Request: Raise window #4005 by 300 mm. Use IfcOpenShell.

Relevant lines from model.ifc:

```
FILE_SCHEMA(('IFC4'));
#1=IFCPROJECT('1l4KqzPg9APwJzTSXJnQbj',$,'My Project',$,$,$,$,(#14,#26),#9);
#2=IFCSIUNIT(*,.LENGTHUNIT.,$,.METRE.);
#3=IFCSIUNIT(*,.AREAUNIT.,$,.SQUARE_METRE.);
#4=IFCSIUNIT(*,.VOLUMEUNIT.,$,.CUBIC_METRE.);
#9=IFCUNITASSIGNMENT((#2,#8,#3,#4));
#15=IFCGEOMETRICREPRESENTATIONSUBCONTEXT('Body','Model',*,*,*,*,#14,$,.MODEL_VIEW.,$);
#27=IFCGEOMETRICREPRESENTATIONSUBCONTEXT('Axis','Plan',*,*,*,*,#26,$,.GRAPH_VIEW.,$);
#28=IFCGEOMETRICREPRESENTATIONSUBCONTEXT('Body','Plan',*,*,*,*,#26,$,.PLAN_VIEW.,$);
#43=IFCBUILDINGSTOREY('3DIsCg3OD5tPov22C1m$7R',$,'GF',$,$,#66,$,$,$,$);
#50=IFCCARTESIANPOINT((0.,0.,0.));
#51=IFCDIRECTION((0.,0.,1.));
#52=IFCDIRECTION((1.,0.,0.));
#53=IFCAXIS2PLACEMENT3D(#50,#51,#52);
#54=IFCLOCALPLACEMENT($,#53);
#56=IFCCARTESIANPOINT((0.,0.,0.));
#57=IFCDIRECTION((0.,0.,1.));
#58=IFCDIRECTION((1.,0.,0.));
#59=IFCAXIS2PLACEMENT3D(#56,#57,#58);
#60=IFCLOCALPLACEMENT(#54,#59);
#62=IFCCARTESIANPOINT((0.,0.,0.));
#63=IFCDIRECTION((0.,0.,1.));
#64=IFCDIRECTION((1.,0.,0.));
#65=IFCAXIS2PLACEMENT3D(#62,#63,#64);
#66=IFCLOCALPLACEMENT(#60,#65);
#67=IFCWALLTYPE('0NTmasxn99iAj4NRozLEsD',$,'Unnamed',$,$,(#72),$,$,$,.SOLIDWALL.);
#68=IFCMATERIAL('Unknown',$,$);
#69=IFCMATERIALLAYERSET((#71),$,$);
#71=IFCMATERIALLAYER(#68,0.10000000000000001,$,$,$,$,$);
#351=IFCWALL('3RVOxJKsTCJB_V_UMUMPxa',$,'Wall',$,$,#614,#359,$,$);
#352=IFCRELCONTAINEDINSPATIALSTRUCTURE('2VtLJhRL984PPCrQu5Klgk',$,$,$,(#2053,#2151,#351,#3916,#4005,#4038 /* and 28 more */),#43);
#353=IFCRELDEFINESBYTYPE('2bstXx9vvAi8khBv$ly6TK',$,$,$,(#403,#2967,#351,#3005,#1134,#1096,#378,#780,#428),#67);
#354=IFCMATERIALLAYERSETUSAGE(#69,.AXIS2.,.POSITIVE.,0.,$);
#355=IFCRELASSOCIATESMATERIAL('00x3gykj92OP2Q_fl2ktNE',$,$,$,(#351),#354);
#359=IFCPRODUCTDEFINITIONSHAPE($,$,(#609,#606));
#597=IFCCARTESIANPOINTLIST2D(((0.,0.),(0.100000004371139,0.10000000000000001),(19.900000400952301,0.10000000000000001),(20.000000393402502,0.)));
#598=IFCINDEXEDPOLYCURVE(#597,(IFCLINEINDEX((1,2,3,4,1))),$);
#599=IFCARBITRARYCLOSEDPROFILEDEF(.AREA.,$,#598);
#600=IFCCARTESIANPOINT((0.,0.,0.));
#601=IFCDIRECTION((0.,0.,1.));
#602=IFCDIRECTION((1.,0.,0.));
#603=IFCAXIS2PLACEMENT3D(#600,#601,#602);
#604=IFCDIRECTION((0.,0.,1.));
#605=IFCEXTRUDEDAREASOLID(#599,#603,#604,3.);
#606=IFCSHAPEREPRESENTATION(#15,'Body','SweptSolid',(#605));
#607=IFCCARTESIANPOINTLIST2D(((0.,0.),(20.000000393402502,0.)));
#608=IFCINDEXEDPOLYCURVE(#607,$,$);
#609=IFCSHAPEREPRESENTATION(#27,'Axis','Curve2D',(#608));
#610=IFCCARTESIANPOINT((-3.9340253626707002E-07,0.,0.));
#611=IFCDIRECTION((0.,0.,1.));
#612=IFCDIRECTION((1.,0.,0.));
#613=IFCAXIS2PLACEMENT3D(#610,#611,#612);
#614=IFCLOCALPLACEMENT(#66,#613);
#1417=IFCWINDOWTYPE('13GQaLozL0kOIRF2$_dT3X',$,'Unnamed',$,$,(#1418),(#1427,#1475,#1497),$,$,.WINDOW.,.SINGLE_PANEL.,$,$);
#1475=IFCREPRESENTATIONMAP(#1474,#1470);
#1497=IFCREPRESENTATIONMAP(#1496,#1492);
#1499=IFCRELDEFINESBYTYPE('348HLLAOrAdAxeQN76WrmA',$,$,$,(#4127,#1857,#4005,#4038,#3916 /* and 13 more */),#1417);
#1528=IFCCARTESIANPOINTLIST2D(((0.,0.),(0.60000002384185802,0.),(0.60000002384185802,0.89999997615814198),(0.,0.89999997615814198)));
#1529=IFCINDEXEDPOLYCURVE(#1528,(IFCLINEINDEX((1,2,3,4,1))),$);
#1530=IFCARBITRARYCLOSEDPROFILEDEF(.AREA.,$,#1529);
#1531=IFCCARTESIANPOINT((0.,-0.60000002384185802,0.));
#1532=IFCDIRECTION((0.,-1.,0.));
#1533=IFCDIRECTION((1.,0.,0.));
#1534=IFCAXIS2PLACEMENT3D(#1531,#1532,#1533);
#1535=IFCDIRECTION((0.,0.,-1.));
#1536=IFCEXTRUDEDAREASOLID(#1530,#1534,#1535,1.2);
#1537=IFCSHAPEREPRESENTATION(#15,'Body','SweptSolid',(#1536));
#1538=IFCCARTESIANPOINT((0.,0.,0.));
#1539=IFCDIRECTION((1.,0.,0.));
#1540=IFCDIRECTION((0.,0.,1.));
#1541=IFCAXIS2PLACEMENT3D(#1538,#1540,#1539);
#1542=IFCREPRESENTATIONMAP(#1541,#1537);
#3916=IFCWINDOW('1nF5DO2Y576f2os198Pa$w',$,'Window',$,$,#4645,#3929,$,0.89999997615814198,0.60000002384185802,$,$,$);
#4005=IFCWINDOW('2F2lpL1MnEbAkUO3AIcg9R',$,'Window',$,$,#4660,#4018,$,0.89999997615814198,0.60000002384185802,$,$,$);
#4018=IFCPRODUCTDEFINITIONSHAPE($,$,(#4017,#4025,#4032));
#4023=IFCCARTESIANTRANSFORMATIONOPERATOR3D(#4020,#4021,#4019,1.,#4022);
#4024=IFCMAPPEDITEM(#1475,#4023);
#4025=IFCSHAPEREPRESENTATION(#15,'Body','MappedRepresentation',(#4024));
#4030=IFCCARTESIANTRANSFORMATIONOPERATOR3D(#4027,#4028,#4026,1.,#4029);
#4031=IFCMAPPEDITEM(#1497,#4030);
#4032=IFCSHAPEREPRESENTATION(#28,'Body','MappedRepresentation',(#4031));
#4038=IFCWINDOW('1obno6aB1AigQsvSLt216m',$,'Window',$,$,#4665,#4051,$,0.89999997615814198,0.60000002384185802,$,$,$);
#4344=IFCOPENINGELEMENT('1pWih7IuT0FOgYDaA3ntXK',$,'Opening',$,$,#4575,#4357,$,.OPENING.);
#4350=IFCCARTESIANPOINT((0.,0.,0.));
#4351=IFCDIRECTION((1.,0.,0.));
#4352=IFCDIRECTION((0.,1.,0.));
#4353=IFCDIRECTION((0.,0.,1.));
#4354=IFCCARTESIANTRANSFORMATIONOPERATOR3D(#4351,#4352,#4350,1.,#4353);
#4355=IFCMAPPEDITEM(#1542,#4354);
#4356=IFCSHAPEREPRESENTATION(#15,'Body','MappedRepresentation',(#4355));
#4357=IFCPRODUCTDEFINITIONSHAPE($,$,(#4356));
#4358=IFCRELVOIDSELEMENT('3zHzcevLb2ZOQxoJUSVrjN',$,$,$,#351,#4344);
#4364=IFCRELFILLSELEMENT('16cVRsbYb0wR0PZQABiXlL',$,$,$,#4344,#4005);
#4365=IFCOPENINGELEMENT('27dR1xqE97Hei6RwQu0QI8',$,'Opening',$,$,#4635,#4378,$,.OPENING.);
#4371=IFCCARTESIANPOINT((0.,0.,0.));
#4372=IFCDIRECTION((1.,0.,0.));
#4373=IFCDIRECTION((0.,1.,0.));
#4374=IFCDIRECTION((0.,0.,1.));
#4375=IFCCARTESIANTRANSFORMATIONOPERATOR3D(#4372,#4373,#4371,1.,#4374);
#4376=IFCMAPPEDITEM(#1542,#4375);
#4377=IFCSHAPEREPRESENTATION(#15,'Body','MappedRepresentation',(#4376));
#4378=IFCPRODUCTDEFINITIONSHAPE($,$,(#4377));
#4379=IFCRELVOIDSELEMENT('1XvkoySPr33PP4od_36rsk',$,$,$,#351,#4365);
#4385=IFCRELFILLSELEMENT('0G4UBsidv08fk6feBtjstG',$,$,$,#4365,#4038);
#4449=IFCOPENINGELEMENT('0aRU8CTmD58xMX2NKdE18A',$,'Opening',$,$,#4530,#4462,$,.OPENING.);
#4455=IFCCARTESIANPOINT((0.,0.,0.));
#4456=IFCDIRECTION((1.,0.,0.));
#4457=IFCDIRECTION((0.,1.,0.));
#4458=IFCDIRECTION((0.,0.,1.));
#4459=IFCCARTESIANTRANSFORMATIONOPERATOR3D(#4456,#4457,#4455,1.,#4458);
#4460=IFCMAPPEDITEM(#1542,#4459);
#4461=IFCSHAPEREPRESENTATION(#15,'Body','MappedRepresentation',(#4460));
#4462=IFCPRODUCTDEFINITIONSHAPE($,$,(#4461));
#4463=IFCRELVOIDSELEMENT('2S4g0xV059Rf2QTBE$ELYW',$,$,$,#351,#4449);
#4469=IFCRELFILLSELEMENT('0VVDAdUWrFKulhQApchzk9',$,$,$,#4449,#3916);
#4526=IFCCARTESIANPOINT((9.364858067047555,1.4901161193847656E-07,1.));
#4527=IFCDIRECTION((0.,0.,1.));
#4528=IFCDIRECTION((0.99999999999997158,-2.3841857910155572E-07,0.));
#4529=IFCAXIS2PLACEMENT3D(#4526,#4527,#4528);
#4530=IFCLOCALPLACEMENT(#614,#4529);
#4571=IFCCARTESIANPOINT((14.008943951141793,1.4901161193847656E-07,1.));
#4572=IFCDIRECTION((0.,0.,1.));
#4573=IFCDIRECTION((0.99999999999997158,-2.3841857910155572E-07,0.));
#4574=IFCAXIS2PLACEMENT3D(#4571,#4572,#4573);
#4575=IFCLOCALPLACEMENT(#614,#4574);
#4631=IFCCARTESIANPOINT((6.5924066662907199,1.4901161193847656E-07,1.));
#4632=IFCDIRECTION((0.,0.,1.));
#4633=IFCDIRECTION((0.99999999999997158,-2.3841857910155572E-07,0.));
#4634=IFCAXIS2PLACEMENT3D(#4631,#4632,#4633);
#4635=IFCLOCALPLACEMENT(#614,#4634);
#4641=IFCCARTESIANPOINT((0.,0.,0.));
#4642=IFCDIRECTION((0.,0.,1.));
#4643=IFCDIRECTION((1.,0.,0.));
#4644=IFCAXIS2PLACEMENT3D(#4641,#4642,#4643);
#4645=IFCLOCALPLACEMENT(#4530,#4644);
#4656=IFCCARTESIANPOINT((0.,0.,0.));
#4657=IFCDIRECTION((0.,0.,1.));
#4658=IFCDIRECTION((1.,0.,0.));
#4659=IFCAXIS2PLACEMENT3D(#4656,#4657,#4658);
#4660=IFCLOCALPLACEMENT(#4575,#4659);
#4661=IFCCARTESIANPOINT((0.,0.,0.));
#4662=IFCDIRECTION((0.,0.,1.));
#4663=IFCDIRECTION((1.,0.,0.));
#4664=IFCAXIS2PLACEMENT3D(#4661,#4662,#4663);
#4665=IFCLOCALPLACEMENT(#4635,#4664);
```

```python
import numpy as np
import ifcopenshell
import ifcopenshell.api.geometry
import ifcopenshell.util.placement
import ifcopenshell.util.unit

model = ifcopenshell.open("model.ifc")
unit_scale = ifcopenshell.util.unit.calculate_unit_scale(model)

window = model.by_guid("2F2lpL1MnEbAkUO3AIcg9R")
opening = window.FillsVoids[0].RelatingOpeningElement
dz = 0.3 / unit_scale

shift = np.array([0.0, 0.0, dz])
# The window is placed relative to its opening, so it follows when the opening moves.
matrix = ifcopenshell.util.placement.get_local_placement(opening.ObjectPlacement)
matrix[:3, 3] += shift
ifcopenshell.api.geometry.edit_object_placement(
    model, product=opening, matrix=matrix, is_si=False, should_transform_children=True
)

print(f"moved by {dz * unit_scale:+.3f} m")

model.write("model_edited.ifc")
```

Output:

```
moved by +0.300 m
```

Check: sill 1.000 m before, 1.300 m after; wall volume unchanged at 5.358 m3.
